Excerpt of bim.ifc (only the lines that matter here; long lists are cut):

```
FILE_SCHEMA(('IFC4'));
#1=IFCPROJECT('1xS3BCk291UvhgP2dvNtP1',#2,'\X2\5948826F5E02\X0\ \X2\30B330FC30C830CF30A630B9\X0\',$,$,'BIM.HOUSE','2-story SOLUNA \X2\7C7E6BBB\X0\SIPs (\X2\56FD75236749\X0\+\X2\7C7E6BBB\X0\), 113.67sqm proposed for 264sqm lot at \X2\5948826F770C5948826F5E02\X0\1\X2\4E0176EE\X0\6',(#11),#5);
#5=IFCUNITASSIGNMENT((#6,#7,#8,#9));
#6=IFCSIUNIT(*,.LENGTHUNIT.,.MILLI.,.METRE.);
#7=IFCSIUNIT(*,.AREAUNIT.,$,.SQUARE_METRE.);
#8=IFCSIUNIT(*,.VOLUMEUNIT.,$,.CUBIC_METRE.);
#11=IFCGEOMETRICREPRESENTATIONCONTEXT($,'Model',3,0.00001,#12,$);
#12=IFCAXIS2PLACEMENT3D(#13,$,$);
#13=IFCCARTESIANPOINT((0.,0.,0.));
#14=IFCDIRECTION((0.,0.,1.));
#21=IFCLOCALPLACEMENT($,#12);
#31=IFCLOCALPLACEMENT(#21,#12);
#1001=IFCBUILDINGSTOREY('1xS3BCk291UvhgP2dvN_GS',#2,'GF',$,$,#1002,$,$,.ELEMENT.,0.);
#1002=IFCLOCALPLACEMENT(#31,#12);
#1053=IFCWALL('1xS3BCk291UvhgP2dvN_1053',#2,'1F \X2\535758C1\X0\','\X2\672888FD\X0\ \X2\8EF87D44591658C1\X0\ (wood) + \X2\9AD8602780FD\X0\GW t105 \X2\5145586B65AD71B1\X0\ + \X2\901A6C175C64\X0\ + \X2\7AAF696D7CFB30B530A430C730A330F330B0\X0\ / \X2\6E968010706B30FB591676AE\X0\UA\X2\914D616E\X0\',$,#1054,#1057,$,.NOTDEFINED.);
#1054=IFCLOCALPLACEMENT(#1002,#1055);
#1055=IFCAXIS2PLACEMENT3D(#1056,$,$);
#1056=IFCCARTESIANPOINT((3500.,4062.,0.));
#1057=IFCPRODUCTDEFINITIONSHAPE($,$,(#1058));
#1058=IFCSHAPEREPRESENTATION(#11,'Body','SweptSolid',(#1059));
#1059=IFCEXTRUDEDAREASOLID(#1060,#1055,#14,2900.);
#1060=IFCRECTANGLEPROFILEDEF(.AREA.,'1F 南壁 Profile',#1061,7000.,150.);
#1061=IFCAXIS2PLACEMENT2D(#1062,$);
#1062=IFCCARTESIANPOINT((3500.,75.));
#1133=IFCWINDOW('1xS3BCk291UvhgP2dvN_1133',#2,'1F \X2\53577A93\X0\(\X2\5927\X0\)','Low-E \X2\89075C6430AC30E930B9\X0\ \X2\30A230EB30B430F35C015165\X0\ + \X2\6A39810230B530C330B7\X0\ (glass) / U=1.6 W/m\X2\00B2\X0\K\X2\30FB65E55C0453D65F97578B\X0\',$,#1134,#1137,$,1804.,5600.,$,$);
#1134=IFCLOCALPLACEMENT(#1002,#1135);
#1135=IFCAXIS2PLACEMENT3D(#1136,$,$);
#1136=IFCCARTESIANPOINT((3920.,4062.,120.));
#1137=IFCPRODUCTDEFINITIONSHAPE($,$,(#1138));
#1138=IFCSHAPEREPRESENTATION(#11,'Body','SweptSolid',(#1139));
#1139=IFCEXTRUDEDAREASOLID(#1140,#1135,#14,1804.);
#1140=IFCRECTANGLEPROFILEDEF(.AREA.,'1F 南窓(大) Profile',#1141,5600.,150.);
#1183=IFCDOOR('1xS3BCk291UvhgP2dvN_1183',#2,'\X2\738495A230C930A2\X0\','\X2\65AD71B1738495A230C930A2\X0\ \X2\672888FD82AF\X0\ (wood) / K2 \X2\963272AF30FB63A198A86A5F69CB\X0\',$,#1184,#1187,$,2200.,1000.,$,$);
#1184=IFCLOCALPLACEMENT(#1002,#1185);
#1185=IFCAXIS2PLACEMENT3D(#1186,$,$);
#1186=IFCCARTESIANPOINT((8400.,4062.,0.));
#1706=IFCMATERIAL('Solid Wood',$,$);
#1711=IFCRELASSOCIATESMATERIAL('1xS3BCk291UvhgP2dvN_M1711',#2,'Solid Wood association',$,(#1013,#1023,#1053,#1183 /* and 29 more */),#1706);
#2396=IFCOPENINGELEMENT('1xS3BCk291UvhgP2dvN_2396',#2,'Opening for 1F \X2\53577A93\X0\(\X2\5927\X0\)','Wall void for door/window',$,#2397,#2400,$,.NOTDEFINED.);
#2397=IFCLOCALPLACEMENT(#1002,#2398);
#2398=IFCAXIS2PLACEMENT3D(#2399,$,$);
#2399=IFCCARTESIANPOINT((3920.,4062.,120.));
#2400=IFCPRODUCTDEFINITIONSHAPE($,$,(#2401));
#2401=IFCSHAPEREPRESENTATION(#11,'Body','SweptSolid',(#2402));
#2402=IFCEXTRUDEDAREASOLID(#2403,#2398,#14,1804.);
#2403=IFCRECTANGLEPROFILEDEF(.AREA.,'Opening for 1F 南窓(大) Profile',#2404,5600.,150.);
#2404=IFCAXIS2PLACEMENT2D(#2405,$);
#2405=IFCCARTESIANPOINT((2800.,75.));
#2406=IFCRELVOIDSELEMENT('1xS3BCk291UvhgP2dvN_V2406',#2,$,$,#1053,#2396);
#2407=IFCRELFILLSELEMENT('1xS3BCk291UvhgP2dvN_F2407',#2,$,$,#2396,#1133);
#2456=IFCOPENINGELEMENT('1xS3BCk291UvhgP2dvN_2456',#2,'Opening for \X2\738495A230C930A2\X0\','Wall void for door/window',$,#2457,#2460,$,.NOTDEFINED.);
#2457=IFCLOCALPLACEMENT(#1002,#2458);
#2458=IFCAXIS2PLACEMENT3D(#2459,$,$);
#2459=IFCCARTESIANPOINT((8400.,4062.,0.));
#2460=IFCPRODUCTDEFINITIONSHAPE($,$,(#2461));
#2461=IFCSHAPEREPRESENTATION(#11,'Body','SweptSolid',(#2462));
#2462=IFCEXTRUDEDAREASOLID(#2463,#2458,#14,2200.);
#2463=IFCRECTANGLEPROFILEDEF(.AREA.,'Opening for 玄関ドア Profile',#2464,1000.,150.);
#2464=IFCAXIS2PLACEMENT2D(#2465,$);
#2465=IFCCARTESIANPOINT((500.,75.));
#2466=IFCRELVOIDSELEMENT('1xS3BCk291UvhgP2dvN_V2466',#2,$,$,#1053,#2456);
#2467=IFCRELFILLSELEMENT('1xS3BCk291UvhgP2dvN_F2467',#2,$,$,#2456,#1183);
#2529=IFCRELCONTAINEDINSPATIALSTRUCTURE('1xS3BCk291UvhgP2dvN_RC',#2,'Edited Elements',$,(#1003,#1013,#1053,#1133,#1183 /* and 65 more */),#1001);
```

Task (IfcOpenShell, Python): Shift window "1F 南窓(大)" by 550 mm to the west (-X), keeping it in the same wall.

```python
import ifcopenshell
import ifcopenshell.api.geometry
import ifcopenshell.util.placement
import ifcopenshell.util.unit

model = ifcopenshell.open("bim.ifc")
unit_scale = ifcopenshell.util.unit.calculate_unit_scale(model)

window = model.by_guid("1xS3BCk291UvhgP2dvN_1133")
opening = window.FillsVoids[0].RelatingOpeningElement
wall = opening.VoidsElements[0].RelatingBuildingElement

wall_matrix = ifcopenshell.util.placement.get_local_placement(wall.ObjectPlacement)
shift = wall_matrix[:3, 0] * -0.55 / unit_scale
before = ifcopenshell.util.placement.get_local_placement(window.ObjectPlacement)[:3, 3].copy()

# The window is not placed relative to its opening, so move both.
for product in (opening, window):
    matrix = ifcopenshell.util.placement.get_local_placement(product.ObjectPlacement)
    matrix[:3, 3] += shift
    ifcopenshell.api.geometry.edit_object_placement(model, product=product, matrix=matrix, is_si=False)

after = ifcopenshell.util.placement.get_local_placement(window.ObjectPlacement)[:3, 3]
print("window moved by", (after - before).round(3) + 0.0)

model.write("bim_rev.ifc")
```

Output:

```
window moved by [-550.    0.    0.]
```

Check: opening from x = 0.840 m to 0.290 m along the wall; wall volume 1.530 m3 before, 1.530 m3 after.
